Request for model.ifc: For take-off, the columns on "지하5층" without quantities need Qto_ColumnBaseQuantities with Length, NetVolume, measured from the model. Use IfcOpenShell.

First a look at what the model holds.

```python
import ifcopenshell
import ifcopenshell.util.element
import ifcopenshell.util.unit

model = ifcopenshell.open("model.ifc")
print(model.schema)
for unit_type in ("LENGTHUNIT", "AREAUNIT", "VOLUMEUNIT"):
    print(unit_type, ifcopenshell.util.unit.calculate_unit_scale(model, unit_type))
storey = next(s for s in model.by_type("IfcBuildingStorey") if s.Name == "지하5층")
columns = [e for e in ifcopenshell.util.element.get_decomposition(storey) if e.is_a("IfcColumn")]
for e in sorted(columns, key=lambda e: e.id()):
    print(e.id(), e.is_a(), e.Name, list(ifcopenshell.util.element.get_psets(e, qtos_only=True)), sep=" | ")
```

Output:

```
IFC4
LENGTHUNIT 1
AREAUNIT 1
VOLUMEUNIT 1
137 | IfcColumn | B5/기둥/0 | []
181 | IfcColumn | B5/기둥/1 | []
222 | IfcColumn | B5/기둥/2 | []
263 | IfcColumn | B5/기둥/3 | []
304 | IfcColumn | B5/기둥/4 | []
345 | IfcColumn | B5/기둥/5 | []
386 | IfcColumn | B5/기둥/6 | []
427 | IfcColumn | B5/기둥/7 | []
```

```python
import ifcopenshell
import ifcopenshell.api.pset
import ifcopenshell.geom
import ifcopenshell.util.element
import ifcopenshell.util.shape
import ifcopenshell.util.unit

model = ifcopenshell.open("model.ifc")
unit_scale = ifcopenshell.util.unit.calculate_unit_scale(model)
volume_scale = ifcopenshell.util.unit.calculate_unit_scale(model, "VOLUMEUNIT")
settings = ifcopenshell.geom.settings()

storey = next(s for s in model.by_type("IfcBuildingStorey") if s.Name == "지하5층")
columns = [e for e in ifcopenshell.util.element.get_decomposition(storey) if e.is_a("IfcColumn")]

for e in sorted(columns, key=lambda e: e.id()):
    if ifcopenshell.util.element.get_psets(e, qtos_only=True, should_inherit=False):
        continue
    # Geometry comes back in metres, in the element's own axes.
    shape = ifcopenshell.geom.create_shape(settings, e)
    values = {
        "Length": ifcopenshell.util.shape.get_z(shape.geometry) / unit_scale,
        "NetVolume": ifcopenshell.util.shape.get_volume(shape.geometry) / volume_scale,
    }
    qto = ifcopenshell.api.pset.add_qto(model, product=e, name="Qto_ColumnBaseQuantities")
    ifcopenshell.api.pset.edit_qto(model, qto=qto, properties=values)
    print(e.id(), {k: round(v, 3) for k, v in values.items()})

model.write("model-out.ifc")
```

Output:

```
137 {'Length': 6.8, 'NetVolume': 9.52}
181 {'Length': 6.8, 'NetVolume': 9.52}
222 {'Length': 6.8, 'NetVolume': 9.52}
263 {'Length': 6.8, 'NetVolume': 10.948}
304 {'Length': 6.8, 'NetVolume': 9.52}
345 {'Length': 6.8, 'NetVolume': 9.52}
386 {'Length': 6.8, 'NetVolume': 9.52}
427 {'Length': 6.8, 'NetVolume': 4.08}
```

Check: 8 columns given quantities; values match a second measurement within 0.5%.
